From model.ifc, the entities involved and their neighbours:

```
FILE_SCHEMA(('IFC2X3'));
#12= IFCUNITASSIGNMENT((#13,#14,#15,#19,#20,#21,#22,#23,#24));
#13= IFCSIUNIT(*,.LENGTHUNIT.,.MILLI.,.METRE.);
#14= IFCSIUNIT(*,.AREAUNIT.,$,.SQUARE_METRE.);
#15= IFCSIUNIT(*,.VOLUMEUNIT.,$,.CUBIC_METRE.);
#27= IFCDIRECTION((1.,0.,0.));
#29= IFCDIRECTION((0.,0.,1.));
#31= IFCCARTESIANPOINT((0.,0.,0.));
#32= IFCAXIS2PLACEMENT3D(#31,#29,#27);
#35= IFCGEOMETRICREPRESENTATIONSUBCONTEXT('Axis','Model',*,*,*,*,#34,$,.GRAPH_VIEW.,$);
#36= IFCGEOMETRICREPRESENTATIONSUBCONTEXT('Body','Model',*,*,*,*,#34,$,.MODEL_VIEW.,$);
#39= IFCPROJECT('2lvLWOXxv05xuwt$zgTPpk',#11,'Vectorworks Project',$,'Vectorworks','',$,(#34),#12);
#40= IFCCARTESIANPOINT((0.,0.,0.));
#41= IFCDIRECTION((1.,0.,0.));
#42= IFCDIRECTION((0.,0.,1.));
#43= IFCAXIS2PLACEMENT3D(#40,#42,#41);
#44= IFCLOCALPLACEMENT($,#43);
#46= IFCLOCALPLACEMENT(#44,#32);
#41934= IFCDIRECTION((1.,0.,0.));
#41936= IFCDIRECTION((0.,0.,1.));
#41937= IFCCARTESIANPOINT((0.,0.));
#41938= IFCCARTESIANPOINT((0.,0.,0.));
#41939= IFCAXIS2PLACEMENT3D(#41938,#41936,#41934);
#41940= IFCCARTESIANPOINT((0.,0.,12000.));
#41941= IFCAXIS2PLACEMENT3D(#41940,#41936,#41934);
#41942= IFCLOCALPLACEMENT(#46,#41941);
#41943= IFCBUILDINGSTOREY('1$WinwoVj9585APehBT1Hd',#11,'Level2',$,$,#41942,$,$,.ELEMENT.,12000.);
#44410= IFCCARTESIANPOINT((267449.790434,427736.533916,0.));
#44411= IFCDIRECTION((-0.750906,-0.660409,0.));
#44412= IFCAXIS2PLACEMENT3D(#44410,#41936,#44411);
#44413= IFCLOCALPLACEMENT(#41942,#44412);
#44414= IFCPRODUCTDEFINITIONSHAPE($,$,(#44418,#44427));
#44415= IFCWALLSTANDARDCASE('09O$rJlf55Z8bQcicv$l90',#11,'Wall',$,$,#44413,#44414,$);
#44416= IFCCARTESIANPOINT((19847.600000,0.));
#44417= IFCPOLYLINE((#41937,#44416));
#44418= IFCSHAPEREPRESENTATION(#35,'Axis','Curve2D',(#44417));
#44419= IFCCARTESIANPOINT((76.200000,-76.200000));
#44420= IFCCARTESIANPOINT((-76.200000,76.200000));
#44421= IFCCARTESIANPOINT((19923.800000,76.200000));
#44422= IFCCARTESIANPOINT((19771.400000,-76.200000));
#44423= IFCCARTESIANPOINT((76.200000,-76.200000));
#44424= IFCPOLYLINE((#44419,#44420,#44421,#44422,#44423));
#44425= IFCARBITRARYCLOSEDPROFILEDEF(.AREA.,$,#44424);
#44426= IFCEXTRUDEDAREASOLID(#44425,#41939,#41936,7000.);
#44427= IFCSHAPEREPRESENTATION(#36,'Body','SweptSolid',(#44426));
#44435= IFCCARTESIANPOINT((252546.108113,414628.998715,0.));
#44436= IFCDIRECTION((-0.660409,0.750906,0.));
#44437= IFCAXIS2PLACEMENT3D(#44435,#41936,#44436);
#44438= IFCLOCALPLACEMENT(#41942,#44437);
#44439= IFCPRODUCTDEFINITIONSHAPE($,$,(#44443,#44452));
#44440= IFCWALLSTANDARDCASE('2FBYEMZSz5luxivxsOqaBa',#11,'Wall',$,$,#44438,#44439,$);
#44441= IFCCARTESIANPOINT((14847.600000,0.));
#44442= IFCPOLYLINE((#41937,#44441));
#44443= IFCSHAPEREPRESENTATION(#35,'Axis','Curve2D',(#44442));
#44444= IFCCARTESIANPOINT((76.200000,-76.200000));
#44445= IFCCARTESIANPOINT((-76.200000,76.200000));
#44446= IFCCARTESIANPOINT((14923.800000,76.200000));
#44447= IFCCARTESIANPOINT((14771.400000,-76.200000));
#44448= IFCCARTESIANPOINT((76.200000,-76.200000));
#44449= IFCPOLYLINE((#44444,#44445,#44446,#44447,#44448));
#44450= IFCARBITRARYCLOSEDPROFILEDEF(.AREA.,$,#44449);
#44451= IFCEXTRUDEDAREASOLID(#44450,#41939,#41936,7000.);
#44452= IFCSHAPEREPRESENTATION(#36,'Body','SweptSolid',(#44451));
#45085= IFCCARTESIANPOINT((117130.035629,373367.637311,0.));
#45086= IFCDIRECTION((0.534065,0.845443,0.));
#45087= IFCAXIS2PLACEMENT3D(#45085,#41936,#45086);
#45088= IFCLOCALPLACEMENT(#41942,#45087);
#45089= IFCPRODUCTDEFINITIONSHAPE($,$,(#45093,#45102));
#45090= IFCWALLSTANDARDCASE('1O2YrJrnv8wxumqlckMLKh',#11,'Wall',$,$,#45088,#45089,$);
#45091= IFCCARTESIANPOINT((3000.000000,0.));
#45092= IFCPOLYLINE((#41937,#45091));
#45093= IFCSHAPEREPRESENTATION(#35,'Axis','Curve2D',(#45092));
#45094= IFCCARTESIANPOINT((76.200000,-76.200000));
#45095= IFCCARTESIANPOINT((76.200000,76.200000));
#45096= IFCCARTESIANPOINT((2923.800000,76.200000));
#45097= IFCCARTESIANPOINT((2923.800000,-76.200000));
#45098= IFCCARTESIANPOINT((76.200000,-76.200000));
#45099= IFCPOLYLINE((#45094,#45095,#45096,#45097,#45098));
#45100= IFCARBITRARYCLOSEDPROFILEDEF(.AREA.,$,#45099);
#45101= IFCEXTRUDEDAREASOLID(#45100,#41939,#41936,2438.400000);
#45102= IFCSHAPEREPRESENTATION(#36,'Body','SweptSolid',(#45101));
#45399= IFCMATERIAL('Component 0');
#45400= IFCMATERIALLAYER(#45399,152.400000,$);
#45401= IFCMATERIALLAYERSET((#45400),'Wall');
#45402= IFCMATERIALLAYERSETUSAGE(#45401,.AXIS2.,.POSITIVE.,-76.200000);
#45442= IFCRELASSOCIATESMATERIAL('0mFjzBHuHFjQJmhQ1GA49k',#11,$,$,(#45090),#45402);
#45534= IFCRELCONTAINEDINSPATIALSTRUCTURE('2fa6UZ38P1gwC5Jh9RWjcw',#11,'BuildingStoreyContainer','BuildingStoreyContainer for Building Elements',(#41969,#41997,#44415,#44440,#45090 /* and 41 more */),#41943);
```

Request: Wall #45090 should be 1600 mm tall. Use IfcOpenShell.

```python
import ifcopenshell
import ifcopenshell.geom
import ifcopenshell.util.representation
import ifcopenshell.util.shape
import ifcopenshell.util.unit

model = ifcopenshell.open("model.ifc")
unit_scale = ifcopenshell.util.unit.calculate_unit_scale(model)
settings = ifcopenshell.geom.settings()


def volume(element):
    """Net volume in cubic metres, openings subtracted."""
    shape = ifcopenshell.geom.create_shape(settings, element)
    return ifcopenshell.util.shape.get_volume(shape.geometry)


wall = model.by_guid("1O2YrJrnv8wxumqlckMLKh")
before = volume(wall)

body = ifcopenshell.util.representation.get_representation(wall, "Model", "Body")
solid = body.Items[0]
old_height = solid.Depth
solid.Depth = 1.6 / unit_scale
after = volume(wall)

print(f"height {old_height:g} -> {solid.Depth:g}, volume {before:.3f} -> {after:.3f} m3")

model.write("model_updated.ifc")
```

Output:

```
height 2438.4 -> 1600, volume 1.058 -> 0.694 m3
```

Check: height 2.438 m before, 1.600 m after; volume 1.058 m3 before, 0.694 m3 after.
